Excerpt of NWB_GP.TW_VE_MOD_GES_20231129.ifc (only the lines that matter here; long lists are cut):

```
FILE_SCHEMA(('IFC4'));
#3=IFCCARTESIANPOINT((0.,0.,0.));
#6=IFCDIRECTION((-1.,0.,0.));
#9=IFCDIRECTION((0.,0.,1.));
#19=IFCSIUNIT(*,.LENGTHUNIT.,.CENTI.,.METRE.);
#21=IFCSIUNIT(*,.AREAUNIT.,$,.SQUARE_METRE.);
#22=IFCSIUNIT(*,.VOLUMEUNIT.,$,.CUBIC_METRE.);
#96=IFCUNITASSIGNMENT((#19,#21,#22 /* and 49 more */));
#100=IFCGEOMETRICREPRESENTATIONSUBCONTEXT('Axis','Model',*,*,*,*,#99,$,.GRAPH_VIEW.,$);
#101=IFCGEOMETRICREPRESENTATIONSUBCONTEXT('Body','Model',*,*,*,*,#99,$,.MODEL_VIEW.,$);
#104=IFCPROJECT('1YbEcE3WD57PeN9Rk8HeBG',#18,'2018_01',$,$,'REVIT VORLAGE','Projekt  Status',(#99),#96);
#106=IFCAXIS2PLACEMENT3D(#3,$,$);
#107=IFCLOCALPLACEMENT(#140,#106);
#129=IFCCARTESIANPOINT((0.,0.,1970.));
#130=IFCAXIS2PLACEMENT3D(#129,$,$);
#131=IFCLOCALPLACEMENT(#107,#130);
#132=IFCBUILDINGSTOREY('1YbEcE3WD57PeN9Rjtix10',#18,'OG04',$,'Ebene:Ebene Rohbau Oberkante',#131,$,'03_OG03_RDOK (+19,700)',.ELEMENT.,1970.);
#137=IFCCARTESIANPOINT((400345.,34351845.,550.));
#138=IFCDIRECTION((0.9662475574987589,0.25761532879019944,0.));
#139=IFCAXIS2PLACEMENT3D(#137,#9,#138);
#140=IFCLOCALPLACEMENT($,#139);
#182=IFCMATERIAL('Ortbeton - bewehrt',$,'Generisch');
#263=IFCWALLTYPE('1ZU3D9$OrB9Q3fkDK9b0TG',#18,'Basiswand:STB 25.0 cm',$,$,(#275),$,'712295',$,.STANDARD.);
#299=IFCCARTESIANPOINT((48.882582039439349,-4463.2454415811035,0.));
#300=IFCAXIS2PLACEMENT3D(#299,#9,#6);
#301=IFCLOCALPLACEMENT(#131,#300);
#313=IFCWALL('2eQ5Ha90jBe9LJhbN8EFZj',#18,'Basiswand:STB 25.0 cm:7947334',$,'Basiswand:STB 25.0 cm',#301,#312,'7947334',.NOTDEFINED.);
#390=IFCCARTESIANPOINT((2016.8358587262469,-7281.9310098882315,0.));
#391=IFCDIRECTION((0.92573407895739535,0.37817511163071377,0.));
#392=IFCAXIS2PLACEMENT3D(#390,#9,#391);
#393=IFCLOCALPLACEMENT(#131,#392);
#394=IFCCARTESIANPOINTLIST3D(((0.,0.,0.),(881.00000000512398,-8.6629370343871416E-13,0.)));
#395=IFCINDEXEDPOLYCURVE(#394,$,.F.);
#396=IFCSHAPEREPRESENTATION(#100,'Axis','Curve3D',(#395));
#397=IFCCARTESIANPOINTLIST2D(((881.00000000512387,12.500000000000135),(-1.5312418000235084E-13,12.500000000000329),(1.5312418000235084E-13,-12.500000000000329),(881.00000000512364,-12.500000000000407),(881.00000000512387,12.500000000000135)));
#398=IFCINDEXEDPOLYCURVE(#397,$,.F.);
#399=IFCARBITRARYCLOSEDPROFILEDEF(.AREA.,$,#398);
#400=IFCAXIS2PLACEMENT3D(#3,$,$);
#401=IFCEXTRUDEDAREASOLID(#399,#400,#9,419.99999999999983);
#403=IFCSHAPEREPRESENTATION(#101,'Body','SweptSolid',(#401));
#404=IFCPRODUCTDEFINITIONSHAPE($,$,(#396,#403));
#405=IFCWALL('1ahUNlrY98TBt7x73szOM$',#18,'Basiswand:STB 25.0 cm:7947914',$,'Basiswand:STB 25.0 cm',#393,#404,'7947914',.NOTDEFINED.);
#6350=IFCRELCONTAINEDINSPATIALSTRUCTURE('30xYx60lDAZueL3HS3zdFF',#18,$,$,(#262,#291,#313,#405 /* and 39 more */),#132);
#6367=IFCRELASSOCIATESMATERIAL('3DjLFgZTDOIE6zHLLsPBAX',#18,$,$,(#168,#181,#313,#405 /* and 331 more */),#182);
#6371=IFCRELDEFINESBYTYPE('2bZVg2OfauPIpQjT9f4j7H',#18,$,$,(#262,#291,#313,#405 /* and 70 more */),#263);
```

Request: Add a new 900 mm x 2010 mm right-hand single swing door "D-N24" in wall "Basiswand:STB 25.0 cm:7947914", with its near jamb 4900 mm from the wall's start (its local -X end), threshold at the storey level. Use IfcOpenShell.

```python
import numpy as np
import ifcopenshell
import ifcopenshell.api.feature
import ifcopenshell.api.geometry
import ifcopenshell.api.root
import ifcopenshell.api.spatial
import ifcopenshell.geom
import ifcopenshell.util.element
import ifcopenshell.util.placement
import ifcopenshell.util.representation
import ifcopenshell.util.shape
import ifcopenshell.util.unit

model = ifcopenshell.open("NWB_GP.TW_VE_MOD_GES_20231129.ifc")
unit_scale = ifcopenshell.util.unit.calculate_unit_scale(model)
settings = ifcopenshell.geom.settings()


def volume(element):
    """Net volume in cubic metres, openings subtracted."""
    shape = ifcopenshell.geom.create_shape(settings, element)
    return ifcopenshell.util.shape.get_volume(shape.geometry)


wall = model.by_id(405)
storey = ifcopenshell.util.element.get_container(wall, ifc_class="IfcBuildingStorey")
context = ifcopenshell.util.representation.get_context(model, "Model", "Body", "MODEL_VIEW")
before = volume(wall)

width, height, from_end, sill = 0.9, 2.01, 4.9, 0.0  # metres

# The wall runs along its own X axis, and the end named is its -X end.
wall_shape = ifcopenshell.geom.create_shape(settings, wall)
x, y, z = ifcopenshell.util.shape.get_vertices(wall_shape.geometry).T
start = x.min() + from_end
face, thickness = float(y.min()), float(y.max() - y.min())
wall_matrix = ifcopenshell.util.placement.get_local_placement(wall.ObjectPlacement)
level = ifcopenshell.util.placement.get_local_placement(storey.ObjectPlacement)[2, 3]


def in_wall(x, y):
    """Placement at x, y metres in the wall's axes, at sill height."""
    matrix = wall_matrix.copy()
    matrix[:, 3] = wall_matrix @ np.array([x / unit_scale, y / unit_scale, 0.0, 1.0])
    matrix[2, 3] = level + sill / unit_scale
    return matrix


# Opening: a box that overshoots both wall faces by 50 mm.
opening = ifcopenshell.api.root.create_entity(model, ifc_class="IfcOpeningElement", predefined_type="OPENING")
box = ifcopenshell.api.geometry.add_wall_representation(
    model, context=context, length=width, height=height, thickness=thickness + 0.1
)
ifcopenshell.api.geometry.assign_representation(model, product=opening, representation=box)
ifcopenshell.api.geometry.edit_object_placement(model, product=opening, matrix=in_wall(start, face - 0.05), is_si=False)
ifcopenshell.api.feature.add_feature(model, feature=opening, element=wall)

door = ifcopenshell.api.root.create_entity(model, ifc_class="IfcDoor", name="D-N24", predefined_type="DOOR")
door.OverallWidth, door.OverallHeight = width / unit_scale, height / unit_scale
door.OperationType = "SINGLE_SWING_RIGHT"
body = ifcopenshell.api.geometry.add_door_representation(
    model,
    context=context,
    overall_width=door.OverallWidth,
    overall_height=door.OverallHeight,
    operation_type="SINGLE_SWING_RIGHT",
    lining_properties={"LiningDepth": thickness / unit_scale, "ThresholdDepth": thickness / unit_scale},
)
ifcopenshell.api.geometry.assign_representation(model, product=door, representation=body)
ifcopenshell.api.spatial.assign_container(model, products=[door], relating_structure=storey)
ifcopenshell.api.feature.add_filling(model, opening=opening, element=door)

# The lining spans the wall, so the door starts at the wall face.
ifcopenshell.api.geometry.edit_object_placement(model, product=door, matrix=in_wall(start, face), is_si=False)

after = volume(wall)

print(f"wall volume {before:.3f} -> {after:.3f} m3")

model.write("NWB_GP.TW_VE_MOD_GES_20231129_edited.ifc")
```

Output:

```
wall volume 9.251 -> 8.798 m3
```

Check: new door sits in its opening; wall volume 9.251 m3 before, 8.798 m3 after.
